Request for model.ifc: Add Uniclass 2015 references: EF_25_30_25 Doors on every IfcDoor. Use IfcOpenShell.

First a look at what the model holds.

```python
import ifcopenshell

model = ifcopenshell.open("model.ifc")
print(model.schema)
print("classifications:", [c.Name for c in model.by_type("IfcClassification")])
for ifc_class in ("IfcDoor", "IfcRoof", "IfcStair", "IfcWall", "IfcWindow"):
    print(ifc_class, len(model.by_type(ifc_class)))
```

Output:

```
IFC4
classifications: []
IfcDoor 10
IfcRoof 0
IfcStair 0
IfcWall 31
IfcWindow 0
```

```python
import ifcopenshell
import ifcopenshell.api.classification

model = ifcopenshell.open("model.ifc")

system = ifcopenshell.api.classification.add_classification(model, classification="Uniclass 2015")

codes = {
    "IfcDoor": ("EF_25_30_25", "Doors"),
}
for ifc_class, (code, name) in codes.items():
    products = model.by_type(ifc_class)
    ifcopenshell.api.classification.add_reference(
        model, products=products, classification=system, identification=code, name=name
    )
    print(code, len(products))

model.write("model_rev.ifc")
```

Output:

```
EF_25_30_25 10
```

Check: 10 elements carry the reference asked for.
